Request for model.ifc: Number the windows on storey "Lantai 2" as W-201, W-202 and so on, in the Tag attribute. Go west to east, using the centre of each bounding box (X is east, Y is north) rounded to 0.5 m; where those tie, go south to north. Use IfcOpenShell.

First a look at what the model holds.

```python
import ifcopenshell
import ifcopenshell.util.element
import ifcopenshell.util.placement

model = ifcopenshell.open("model.ifc")
print(model.schema)
storey = next(s for s in model.by_type("IfcBuildingStorey") if s.Name == "Lantai 2")
windows = [e for e in ifcopenshell.util.element.get_decomposition(storey) if e.is_a("IfcWindow")]
for e in sorted(windows, key=lambda e: e.id()):
    origin = ifcopenshell.util.placement.get_local_placement(e.ObjectPlacement)[:3, 3]
    print(e.id(), e.Tag, e.Name, origin.round(2) + 0.0, sep=" | ")
```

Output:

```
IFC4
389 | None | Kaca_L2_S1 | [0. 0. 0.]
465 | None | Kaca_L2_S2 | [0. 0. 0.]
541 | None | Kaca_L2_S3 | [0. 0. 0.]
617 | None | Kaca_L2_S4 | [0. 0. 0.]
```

```python
import ifcopenshell
import ifcopenshell.geom
import ifcopenshell.util.element
import ifcopenshell.util.shape

model = ifcopenshell.open("model.ifc")
settings = ifcopenshell.geom.settings()
settings.set("use-world-coords", True)


def centre(element):
    shape = ifcopenshell.geom.create_shape(settings, element)
    return ifcopenshell.util.shape.get_bbox_centroid(shape.geometry)


storey = next(s for s in model.by_type("IfcBuildingStorey") if s.Name == "Lantai 2")
windows = [e for e in ifcopenshell.util.element.get_decomposition(storey) if e.is_a("IfcWindow")]

# Insertion points can sit at a corner or the storey origin, so sort by the geometry (in metres).
centres = {e: centre(e) for e in windows}
windows.sort(key=lambda e: (round(centres[e][0] / 0.5), centres[e][1]))

for i, e in enumerate(windows, start=1):
    number = f"W-2{i:02d}"
    e.Tag = number
    print(e.id(), number)

model.write("model_updated.ifc")
```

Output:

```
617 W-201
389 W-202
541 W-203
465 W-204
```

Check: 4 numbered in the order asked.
